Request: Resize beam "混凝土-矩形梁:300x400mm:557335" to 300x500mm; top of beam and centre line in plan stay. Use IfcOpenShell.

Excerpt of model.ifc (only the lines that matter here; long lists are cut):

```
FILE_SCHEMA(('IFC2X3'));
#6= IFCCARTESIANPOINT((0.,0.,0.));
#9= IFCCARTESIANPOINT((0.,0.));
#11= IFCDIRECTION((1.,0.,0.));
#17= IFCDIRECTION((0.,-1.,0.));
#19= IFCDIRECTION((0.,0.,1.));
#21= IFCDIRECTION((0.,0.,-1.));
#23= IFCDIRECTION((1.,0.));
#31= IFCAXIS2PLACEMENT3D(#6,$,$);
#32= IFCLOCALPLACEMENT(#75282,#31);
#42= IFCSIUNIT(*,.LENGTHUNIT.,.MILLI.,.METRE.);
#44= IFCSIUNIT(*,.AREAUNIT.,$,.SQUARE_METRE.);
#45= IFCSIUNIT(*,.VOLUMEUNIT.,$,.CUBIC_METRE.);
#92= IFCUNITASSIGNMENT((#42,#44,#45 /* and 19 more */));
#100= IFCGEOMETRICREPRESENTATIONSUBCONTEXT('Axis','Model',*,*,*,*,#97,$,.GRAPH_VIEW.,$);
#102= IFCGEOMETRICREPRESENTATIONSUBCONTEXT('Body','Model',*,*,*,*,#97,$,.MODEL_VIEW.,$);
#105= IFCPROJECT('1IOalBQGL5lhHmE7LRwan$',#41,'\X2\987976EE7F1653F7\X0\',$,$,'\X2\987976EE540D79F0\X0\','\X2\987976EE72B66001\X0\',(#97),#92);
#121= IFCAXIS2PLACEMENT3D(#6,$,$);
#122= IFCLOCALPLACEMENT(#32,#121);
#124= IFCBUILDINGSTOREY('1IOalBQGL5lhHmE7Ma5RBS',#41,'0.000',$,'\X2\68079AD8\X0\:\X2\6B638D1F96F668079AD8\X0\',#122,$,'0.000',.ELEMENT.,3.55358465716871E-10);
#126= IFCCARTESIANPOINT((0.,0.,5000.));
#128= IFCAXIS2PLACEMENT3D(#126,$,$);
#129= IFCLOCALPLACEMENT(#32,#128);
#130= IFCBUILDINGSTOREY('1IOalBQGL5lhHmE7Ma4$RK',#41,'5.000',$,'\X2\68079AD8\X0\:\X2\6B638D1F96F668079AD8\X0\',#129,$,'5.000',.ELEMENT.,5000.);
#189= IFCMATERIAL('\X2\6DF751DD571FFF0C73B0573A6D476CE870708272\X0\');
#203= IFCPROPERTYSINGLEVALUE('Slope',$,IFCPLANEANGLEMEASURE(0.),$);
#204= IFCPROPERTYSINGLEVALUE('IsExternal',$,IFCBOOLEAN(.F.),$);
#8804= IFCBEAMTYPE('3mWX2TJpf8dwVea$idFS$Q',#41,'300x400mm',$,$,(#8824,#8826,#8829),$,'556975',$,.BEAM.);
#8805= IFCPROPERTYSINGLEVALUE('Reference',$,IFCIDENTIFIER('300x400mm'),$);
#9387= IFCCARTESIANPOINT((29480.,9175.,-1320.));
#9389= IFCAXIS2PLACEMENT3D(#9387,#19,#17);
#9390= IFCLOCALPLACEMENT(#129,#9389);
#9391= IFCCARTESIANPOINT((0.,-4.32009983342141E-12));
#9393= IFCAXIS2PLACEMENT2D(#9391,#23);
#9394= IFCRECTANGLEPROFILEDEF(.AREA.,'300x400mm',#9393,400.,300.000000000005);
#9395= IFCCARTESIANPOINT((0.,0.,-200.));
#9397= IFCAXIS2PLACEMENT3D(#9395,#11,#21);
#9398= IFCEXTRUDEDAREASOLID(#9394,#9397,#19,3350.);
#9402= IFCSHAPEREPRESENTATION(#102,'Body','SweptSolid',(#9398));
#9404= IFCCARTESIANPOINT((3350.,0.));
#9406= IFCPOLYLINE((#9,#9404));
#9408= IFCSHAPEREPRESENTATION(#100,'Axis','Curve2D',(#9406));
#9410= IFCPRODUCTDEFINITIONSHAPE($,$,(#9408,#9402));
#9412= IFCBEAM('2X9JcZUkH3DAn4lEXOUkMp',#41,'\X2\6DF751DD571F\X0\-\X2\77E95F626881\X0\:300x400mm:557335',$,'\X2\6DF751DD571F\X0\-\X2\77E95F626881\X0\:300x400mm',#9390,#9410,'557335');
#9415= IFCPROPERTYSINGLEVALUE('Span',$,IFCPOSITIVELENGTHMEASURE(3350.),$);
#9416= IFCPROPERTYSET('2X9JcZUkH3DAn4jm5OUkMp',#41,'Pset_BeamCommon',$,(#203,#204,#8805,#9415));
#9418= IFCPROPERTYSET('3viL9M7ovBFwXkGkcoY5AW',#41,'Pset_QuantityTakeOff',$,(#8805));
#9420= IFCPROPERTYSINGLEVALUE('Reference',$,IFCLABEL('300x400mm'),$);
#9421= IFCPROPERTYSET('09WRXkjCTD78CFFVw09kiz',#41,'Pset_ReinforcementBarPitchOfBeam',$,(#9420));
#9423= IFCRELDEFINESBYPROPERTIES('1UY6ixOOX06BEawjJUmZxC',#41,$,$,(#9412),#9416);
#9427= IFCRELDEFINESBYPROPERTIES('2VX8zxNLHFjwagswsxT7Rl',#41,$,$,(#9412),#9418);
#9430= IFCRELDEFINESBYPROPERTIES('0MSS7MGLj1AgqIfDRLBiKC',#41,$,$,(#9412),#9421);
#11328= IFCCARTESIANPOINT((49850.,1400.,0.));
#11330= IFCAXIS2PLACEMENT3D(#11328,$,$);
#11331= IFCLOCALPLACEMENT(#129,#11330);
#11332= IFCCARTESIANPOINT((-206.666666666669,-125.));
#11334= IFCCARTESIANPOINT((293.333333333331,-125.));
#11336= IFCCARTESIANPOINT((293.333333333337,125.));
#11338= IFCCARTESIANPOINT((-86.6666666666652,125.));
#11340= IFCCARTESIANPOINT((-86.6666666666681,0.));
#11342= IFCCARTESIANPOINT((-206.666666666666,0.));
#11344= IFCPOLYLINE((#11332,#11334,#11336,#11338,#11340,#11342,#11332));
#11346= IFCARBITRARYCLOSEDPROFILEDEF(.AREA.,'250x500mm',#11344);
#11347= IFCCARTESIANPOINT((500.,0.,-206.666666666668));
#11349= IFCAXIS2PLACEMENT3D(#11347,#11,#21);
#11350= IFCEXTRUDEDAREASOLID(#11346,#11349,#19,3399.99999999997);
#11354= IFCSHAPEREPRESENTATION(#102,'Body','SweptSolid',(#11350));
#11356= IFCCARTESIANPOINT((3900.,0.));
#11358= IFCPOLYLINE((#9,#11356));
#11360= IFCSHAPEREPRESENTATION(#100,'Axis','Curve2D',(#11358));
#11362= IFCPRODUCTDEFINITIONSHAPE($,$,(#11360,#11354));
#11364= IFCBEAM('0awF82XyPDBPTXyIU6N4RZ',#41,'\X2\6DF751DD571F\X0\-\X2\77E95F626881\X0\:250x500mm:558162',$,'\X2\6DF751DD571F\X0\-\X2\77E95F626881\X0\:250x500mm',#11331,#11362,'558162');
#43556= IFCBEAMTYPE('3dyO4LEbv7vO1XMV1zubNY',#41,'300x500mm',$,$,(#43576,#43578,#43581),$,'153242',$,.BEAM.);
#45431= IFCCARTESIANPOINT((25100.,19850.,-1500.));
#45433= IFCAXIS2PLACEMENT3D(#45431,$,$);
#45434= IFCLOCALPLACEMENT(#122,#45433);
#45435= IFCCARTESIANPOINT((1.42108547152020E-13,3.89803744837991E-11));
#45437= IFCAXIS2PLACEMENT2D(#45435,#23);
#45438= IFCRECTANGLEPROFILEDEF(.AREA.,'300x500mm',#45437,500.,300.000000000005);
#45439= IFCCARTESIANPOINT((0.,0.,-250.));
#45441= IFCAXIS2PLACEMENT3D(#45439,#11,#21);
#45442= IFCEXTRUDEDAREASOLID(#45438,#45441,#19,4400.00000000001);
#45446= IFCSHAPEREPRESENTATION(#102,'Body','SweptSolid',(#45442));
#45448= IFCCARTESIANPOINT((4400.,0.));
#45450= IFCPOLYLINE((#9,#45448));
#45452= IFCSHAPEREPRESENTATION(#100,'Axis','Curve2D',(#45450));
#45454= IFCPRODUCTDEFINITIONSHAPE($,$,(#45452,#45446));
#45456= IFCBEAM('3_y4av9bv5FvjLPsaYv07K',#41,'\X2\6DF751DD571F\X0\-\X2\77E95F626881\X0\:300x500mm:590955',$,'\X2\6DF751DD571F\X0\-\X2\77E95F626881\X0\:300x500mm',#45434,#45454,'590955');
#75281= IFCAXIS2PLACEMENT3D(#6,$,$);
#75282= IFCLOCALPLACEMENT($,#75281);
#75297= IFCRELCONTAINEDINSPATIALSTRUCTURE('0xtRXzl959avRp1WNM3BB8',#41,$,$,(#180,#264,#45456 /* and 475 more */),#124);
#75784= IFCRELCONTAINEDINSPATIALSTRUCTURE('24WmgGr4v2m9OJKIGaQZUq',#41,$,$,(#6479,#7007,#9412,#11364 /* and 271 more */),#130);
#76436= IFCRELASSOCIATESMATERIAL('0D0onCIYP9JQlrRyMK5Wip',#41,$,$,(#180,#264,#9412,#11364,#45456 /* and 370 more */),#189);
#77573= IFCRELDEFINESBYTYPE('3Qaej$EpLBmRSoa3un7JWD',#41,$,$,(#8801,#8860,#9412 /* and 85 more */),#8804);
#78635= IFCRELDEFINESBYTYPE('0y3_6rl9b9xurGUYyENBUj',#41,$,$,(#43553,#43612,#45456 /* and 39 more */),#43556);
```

```python
import ifcopenshell
import ifcopenshell.api.pset
import ifcopenshell.api.type
import ifcopenshell.util.element
import ifcopenshell.util.representation

model = ifcopenshell.open("model.ifc")

member = model.by_guid("2X9JcZUkH3DAn4lEXOUkMp")
source = next(p for p in model.by_type("IfcRectangleProfileDef") if p.ProfileName == "300x500mm")

body = ifcopenshell.util.representation.get_representation(member, "Model", "Body")
solid = body.Items[0]
old_profile = solid.SweptArea

# Copy the section's sizes but keep this member's own profile position.
profile = ifcopenshell.util.element.copy(model, source)
# Profiles are centred, so shift by half the change in depth to hold the top.
shift = (old_profile.XDim - profile.XDim) / 2
x, y = old_profile.Position.Location.Coordinates
up = (-1.0, 0.0)  # upwards, in the solid's own plane
location = model.createIfcCartesianPoint((x + up[0] * shift, y + up[1] * shift))
profile.Position = model.createIfcAxis2Placement2D(location, old_profile.Position.RefDirection)
solid.SweptArea = profile
if not model.get_total_inverses(old_profile):
    ifcopenshell.util.element.remove_deep2(model, old_profile)

new_type = model.by_guid("3dyO4LEbv7vO1XMV1zubNY")
ifcopenshell.api.type.assign_type(
    model, related_objects=[member], relating_type=new_type, should_map_representations=False
)
member.Name = member.Name.replace("300x400mm", "300x500mm")
member.ObjectType = "混凝土-矩形梁:300x500mm"
pset = model.by_id(ifcopenshell.util.element.get_pset(member, "Pset_BeamCommon", should_inherit=False)["id"])
ifcopenshell.api.pset.edit_pset(model, pset=pset, properties={"Reference": "300x500mm"})
pset = model.by_id(ifcopenshell.util.element.get_pset(member, "Pset_QuantityTakeOff", should_inherit=False)["id"])
ifcopenshell.api.pset.edit_pset(model, pset=pset, properties={"Reference": "300x500mm"})
pset = model.by_id(ifcopenshell.util.element.get_pset(member, "Pset_ReinforcementBarPitchOfBeam", should_inherit=False)["id"])
ifcopenshell.api.pset.edit_pset(model, pset=pset, properties={"Reference": "300x500mm"})

print(solid.SweptArea)

model.write("model_v2.ifc")
```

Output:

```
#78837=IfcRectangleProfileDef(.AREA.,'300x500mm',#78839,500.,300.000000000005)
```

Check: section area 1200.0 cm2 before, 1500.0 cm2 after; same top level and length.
